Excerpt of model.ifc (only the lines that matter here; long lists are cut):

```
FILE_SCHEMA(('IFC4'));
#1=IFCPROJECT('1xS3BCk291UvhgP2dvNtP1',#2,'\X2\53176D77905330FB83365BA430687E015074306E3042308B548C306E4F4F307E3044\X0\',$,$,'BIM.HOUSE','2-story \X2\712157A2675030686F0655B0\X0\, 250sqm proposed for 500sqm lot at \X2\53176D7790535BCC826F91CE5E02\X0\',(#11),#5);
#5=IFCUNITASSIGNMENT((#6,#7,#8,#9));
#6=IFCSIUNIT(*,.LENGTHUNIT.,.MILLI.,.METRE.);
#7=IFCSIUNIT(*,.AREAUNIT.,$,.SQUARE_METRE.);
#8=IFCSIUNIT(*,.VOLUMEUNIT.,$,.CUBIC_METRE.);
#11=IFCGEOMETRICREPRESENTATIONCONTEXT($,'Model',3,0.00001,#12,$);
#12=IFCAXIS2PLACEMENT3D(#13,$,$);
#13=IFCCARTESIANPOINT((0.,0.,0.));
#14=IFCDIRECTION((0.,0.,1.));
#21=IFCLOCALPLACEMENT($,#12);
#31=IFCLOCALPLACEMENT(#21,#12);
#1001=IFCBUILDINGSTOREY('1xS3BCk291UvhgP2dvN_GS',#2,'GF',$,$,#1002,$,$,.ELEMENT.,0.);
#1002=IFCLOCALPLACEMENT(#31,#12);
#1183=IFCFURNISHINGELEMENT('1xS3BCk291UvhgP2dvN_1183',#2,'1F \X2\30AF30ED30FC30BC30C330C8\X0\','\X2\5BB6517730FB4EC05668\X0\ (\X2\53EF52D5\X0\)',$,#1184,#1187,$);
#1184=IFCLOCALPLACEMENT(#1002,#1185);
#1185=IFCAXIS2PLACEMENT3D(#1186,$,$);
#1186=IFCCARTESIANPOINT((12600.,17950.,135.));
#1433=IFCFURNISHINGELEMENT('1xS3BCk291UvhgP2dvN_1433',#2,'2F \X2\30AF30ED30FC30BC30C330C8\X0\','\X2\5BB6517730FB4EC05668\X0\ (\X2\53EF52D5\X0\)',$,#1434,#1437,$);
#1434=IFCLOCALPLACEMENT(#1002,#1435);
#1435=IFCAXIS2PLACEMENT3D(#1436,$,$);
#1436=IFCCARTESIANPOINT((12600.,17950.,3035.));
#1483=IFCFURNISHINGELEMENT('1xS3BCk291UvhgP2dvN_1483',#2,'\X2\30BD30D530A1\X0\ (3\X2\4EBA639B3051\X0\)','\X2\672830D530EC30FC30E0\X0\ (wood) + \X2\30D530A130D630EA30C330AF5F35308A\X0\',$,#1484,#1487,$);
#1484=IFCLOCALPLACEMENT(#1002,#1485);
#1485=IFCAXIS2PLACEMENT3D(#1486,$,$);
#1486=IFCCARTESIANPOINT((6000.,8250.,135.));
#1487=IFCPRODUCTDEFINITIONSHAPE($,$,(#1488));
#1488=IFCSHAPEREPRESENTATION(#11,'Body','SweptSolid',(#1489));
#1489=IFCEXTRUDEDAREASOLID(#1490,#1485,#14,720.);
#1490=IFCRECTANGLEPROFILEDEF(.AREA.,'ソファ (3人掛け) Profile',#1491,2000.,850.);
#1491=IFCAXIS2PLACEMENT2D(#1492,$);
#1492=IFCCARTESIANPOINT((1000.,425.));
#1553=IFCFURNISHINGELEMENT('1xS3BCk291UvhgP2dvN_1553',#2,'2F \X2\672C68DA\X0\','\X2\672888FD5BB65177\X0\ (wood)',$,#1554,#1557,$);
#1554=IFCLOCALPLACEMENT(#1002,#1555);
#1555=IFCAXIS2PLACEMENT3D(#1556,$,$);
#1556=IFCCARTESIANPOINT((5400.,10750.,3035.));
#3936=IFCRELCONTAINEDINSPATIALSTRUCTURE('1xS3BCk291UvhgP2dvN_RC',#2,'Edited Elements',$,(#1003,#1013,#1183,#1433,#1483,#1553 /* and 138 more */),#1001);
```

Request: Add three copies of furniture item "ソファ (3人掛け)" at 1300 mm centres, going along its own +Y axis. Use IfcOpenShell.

```python
import ifcopenshell
import ifcopenshell.api.geometry
import ifcopenshell.api.root
import ifcopenshell.util.element
import ifcopenshell.util.placement
import ifcopenshell.util.unit

model = ifcopenshell.open("model.ifc")
unit_scale = ifcopenshell.util.unit.calculate_unit_scale(model)


def reuse_history(source, copy):
    """copy_class also copies each property set's owner history, people and application; keep the originals."""
    for rel in copy.IsDefinedBy:
        if rel.is_a("IfcRelDefinesByProperties") and (history := rel.RelatingPropertyDefinition.OwnerHistory):
            rel.RelatingPropertyDefinition.OwnerHistory = source.OwnerHistory
            ifcopenshell.util.element.remove_deep2(model, history)


source = model.by_guid("1xS3BCk291UvhgP2dvN_1483")
base = ifcopenshell.util.placement.get_local_placement(source.ObjectPlacement)
step = base[:3, 1] * 1.3 / unit_scale

for i in range(1, 4):
    copy = ifcopenshell.api.root.copy_class(model, product=source)
    copy.Representation = ifcopenshell.util.element.copy_deep(
        model, source.Representation, exclude=["IfcGeometricRepresentationContext", "IfcRepresentationMap"]
    )
    reuse_history(source, copy)
    matrix = base.copy()
    matrix[:3, 3] += i * step
    print("added at", matrix[:3, 3].round(3) + 0.0)
    ifcopenshell.api.geometry.edit_object_placement(model, product=copy, matrix=matrix, is_si=False)

model.write("model-out.ifc")
```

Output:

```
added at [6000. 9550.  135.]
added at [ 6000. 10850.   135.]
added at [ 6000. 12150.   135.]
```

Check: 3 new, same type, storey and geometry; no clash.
